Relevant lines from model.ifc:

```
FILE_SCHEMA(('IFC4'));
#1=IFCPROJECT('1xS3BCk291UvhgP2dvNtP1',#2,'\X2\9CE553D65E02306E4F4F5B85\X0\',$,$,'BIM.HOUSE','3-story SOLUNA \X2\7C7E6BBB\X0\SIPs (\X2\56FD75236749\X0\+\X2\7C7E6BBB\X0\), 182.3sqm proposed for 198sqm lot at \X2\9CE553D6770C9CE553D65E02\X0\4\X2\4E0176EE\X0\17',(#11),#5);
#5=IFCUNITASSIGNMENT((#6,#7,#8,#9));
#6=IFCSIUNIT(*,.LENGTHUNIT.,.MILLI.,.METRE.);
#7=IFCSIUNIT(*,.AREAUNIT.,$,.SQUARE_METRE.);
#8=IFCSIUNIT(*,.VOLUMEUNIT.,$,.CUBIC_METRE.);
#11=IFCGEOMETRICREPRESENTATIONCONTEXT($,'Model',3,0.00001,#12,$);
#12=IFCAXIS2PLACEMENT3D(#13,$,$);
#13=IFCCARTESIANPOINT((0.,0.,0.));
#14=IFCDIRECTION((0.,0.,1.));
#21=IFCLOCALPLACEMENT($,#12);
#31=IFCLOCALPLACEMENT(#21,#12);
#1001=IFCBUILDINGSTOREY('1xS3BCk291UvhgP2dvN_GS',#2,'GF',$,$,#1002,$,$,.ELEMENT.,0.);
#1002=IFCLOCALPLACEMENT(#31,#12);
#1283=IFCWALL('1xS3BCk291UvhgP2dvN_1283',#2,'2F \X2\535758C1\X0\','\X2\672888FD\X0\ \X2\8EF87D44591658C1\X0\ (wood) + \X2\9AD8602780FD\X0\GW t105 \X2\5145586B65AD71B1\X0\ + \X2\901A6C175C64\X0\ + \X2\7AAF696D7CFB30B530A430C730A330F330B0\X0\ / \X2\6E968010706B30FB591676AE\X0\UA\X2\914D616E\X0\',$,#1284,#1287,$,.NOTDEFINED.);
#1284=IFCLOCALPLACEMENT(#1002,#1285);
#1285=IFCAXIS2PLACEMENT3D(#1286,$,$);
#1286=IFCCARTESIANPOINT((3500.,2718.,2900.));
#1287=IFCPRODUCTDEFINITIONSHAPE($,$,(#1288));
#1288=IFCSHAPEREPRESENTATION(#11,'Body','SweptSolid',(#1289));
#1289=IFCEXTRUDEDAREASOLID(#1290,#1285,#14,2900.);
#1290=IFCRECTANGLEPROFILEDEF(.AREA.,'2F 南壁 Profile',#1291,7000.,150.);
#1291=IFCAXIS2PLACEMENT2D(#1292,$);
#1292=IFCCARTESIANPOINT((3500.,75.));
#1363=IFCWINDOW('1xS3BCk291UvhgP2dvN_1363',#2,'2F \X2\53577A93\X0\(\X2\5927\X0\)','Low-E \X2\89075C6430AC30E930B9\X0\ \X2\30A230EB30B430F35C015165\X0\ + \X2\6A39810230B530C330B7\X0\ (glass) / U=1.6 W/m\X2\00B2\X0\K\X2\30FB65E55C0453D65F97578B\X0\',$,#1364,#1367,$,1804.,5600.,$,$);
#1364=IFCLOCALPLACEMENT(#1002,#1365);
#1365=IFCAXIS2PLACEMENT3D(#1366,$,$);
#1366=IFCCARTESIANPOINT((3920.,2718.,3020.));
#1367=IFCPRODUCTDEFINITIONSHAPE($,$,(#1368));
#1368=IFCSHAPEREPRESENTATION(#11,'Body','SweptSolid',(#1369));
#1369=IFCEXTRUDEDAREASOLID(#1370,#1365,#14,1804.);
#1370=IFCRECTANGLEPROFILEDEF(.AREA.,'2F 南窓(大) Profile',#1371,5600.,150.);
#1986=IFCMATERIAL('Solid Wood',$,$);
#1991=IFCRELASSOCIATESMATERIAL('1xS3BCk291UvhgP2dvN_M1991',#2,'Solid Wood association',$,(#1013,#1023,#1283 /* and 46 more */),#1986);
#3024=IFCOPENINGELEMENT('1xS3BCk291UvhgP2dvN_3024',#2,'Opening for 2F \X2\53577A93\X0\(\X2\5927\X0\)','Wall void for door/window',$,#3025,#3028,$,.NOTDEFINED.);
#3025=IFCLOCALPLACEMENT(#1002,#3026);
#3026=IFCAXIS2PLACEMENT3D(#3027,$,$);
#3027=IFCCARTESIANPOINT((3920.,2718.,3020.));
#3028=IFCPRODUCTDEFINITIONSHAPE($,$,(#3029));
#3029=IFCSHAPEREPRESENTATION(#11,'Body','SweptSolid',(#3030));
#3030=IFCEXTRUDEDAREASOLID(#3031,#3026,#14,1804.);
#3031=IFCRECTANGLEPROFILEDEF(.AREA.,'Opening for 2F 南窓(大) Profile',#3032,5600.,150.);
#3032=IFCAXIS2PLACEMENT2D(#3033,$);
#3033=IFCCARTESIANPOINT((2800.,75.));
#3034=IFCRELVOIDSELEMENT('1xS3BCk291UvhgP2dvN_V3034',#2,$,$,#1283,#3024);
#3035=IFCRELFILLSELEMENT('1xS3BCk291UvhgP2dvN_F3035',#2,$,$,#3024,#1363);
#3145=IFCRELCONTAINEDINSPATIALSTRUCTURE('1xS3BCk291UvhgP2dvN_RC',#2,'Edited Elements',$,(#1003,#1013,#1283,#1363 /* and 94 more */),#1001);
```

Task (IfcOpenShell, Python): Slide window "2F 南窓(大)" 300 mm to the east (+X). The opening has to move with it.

```python
import ifcopenshell
import ifcopenshell.api.geometry
import ifcopenshell.util.placement

model = ifcopenshell.open("model.ifc")

window = model.by_guid("1xS3BCk291UvhgP2dvN_1363")
opening = window.FillsVoids[0].RelatingOpeningElement
wall = opening.VoidsElements[0].RelatingBuildingElement

wall_matrix = ifcopenshell.util.placement.get_local_placement(wall.ObjectPlacement)
shift = wall_matrix[:3, 0] * 300.0
before = ifcopenshell.util.placement.get_local_placement(window.ObjectPlacement)[:3, 3].copy()

# The window is not placed relative to its opening, so move both.
for product in (opening, window):
    matrix = ifcopenshell.util.placement.get_local_placement(product.ObjectPlacement)
    matrix[:3, 3] += shift
    ifcopenshell.api.geometry.edit_object_placement(model, product=product, matrix=matrix, is_si=False)

after = ifcopenshell.util.placement.get_local_placement(window.ObjectPlacement)[:3, 3]
print("window moved by", (after - before).round(3) + 0.0)

model.write("model-out.ifc")
```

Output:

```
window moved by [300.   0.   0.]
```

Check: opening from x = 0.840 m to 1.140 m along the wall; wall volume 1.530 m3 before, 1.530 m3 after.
